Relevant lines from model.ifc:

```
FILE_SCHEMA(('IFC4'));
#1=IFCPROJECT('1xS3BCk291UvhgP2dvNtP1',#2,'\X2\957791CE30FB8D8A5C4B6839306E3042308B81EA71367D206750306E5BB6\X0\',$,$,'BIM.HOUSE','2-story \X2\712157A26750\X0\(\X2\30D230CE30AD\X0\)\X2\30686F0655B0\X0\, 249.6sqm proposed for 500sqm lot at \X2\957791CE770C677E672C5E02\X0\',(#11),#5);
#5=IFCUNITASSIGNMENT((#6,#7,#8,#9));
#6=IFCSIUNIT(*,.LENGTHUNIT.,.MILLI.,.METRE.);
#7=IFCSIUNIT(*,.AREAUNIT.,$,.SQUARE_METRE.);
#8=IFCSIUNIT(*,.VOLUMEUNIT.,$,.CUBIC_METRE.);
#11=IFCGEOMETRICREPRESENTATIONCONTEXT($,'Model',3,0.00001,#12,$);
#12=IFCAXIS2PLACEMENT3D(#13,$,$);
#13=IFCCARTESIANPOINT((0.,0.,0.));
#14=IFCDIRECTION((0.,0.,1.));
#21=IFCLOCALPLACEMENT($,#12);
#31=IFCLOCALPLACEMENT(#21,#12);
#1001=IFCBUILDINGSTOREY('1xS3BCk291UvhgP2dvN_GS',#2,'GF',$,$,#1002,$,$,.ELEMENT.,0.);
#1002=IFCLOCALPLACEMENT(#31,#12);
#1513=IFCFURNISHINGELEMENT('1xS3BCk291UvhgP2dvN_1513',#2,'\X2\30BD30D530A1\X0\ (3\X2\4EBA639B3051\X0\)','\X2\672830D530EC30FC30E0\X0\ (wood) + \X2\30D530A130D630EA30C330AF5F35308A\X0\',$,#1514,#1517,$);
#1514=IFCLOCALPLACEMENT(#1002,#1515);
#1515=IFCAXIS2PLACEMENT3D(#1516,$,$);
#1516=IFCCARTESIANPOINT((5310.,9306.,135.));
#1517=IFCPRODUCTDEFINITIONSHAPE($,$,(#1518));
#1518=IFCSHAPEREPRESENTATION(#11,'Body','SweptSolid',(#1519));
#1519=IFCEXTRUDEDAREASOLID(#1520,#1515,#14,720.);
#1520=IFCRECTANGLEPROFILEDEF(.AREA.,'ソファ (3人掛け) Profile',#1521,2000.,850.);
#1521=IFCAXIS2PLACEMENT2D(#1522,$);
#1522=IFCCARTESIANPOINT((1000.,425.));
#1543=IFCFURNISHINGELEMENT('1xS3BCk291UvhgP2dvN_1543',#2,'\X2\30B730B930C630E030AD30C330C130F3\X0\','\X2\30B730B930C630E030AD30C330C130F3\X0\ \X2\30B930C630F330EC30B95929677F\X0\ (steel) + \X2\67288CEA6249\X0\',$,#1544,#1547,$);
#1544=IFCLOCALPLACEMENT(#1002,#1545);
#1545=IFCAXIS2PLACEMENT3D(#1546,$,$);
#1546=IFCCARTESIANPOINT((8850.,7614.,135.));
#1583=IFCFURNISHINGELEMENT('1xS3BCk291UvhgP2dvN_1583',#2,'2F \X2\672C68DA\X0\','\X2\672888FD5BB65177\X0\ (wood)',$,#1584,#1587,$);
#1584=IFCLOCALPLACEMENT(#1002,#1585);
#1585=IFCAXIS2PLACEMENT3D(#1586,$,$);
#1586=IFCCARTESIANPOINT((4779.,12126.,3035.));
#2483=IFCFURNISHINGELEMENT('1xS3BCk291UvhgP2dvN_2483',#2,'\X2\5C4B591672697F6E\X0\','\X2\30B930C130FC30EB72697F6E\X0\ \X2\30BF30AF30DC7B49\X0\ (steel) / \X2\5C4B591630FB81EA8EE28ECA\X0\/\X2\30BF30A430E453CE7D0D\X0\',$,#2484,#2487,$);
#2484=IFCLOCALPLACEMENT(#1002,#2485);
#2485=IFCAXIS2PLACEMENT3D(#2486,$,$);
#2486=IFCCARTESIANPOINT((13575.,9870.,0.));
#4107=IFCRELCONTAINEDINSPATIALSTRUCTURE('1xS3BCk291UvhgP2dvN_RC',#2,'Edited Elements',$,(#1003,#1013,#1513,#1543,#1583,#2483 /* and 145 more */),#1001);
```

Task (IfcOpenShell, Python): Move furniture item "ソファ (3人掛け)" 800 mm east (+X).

```python
import ifcopenshell
import ifcopenshell.api.geometry
import ifcopenshell.util.placement
import ifcopenshell.util.unit

model = ifcopenshell.open("model.ifc")
unit_scale = ifcopenshell.util.unit.calculate_unit_scale(model)

item = model.by_guid("1xS3BCk291UvhgP2dvN_1513")
matrix = ifcopenshell.util.placement.get_local_placement(item.ObjectPlacement)
matrix[0, 3] += 0.8 / unit_scale
ifcopenshell.api.geometry.edit_object_placement(model, product=item, matrix=matrix, is_si=False)

print(ifcopenshell.util.placement.get_local_placement(item.ObjectPlacement).round(3) + 0.0)

model.write("model_edited.ifc")
```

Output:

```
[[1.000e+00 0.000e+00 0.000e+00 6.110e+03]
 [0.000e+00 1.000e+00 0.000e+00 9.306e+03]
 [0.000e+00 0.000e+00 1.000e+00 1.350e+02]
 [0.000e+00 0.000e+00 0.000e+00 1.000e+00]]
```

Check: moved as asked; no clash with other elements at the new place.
